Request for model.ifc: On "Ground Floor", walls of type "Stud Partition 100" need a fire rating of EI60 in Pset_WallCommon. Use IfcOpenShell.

First a look at what the model holds.

```python
import ifcopenshell
import ifcopenshell.util.element

model = ifcopenshell.open("model.ifc")
print(model.schema)
storey = next(s for s in model.by_type("IfcBuildingStorey") if s.Name == "Ground Floor")
walls = [e for e in ifcopenshell.util.element.get_decomposition(storey) if e.is_a("IfcWall")]
seen = {}
for e in walls:
    element_type = ifcopenshell.util.element.get_type(e)
    key = (element_type.Name if element_type != e and element_type else None, ifcopenshell.util.element.get_pset(e, "Pset_WallCommon", "FireRating"))
    seen[key] = seen.get(key, 0) + 1
for (name, value), count in sorted(seen.items(), key=str):
    print(count, "x", name, "|", value)
```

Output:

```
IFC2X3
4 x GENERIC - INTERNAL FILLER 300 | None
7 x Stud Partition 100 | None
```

```python
import ifcopenshell
import ifcopenshell.api.pset
import ifcopenshell.util.element

model = ifcopenshell.open("model.ifc")

storey = next(s for s in model.by_type("IfcBuildingStorey") if s.Name == "Ground Floor")
walls = [e for e in ifcopenshell.util.element.get_decomposition(storey) if e.is_a("IfcWall")]

count = 0
for e in walls:
    element_type = ifcopenshell.util.element.get_type(e)
    if element_type in (None, e) or element_type.Name != "Stud Partition 100":
        continue
    # add_pset returns the element's existing set when there is one.
    pset = ifcopenshell.api.pset.add_pset(model, product=e, name="Pset_WallCommon")
    ifcopenshell.api.pset.edit_pset(model, pset=pset, properties={"FireRating": "EI60"})
    count += 1

print(count, "walls updated")

model.write("model_edited.ifc")
```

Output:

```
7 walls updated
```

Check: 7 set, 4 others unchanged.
